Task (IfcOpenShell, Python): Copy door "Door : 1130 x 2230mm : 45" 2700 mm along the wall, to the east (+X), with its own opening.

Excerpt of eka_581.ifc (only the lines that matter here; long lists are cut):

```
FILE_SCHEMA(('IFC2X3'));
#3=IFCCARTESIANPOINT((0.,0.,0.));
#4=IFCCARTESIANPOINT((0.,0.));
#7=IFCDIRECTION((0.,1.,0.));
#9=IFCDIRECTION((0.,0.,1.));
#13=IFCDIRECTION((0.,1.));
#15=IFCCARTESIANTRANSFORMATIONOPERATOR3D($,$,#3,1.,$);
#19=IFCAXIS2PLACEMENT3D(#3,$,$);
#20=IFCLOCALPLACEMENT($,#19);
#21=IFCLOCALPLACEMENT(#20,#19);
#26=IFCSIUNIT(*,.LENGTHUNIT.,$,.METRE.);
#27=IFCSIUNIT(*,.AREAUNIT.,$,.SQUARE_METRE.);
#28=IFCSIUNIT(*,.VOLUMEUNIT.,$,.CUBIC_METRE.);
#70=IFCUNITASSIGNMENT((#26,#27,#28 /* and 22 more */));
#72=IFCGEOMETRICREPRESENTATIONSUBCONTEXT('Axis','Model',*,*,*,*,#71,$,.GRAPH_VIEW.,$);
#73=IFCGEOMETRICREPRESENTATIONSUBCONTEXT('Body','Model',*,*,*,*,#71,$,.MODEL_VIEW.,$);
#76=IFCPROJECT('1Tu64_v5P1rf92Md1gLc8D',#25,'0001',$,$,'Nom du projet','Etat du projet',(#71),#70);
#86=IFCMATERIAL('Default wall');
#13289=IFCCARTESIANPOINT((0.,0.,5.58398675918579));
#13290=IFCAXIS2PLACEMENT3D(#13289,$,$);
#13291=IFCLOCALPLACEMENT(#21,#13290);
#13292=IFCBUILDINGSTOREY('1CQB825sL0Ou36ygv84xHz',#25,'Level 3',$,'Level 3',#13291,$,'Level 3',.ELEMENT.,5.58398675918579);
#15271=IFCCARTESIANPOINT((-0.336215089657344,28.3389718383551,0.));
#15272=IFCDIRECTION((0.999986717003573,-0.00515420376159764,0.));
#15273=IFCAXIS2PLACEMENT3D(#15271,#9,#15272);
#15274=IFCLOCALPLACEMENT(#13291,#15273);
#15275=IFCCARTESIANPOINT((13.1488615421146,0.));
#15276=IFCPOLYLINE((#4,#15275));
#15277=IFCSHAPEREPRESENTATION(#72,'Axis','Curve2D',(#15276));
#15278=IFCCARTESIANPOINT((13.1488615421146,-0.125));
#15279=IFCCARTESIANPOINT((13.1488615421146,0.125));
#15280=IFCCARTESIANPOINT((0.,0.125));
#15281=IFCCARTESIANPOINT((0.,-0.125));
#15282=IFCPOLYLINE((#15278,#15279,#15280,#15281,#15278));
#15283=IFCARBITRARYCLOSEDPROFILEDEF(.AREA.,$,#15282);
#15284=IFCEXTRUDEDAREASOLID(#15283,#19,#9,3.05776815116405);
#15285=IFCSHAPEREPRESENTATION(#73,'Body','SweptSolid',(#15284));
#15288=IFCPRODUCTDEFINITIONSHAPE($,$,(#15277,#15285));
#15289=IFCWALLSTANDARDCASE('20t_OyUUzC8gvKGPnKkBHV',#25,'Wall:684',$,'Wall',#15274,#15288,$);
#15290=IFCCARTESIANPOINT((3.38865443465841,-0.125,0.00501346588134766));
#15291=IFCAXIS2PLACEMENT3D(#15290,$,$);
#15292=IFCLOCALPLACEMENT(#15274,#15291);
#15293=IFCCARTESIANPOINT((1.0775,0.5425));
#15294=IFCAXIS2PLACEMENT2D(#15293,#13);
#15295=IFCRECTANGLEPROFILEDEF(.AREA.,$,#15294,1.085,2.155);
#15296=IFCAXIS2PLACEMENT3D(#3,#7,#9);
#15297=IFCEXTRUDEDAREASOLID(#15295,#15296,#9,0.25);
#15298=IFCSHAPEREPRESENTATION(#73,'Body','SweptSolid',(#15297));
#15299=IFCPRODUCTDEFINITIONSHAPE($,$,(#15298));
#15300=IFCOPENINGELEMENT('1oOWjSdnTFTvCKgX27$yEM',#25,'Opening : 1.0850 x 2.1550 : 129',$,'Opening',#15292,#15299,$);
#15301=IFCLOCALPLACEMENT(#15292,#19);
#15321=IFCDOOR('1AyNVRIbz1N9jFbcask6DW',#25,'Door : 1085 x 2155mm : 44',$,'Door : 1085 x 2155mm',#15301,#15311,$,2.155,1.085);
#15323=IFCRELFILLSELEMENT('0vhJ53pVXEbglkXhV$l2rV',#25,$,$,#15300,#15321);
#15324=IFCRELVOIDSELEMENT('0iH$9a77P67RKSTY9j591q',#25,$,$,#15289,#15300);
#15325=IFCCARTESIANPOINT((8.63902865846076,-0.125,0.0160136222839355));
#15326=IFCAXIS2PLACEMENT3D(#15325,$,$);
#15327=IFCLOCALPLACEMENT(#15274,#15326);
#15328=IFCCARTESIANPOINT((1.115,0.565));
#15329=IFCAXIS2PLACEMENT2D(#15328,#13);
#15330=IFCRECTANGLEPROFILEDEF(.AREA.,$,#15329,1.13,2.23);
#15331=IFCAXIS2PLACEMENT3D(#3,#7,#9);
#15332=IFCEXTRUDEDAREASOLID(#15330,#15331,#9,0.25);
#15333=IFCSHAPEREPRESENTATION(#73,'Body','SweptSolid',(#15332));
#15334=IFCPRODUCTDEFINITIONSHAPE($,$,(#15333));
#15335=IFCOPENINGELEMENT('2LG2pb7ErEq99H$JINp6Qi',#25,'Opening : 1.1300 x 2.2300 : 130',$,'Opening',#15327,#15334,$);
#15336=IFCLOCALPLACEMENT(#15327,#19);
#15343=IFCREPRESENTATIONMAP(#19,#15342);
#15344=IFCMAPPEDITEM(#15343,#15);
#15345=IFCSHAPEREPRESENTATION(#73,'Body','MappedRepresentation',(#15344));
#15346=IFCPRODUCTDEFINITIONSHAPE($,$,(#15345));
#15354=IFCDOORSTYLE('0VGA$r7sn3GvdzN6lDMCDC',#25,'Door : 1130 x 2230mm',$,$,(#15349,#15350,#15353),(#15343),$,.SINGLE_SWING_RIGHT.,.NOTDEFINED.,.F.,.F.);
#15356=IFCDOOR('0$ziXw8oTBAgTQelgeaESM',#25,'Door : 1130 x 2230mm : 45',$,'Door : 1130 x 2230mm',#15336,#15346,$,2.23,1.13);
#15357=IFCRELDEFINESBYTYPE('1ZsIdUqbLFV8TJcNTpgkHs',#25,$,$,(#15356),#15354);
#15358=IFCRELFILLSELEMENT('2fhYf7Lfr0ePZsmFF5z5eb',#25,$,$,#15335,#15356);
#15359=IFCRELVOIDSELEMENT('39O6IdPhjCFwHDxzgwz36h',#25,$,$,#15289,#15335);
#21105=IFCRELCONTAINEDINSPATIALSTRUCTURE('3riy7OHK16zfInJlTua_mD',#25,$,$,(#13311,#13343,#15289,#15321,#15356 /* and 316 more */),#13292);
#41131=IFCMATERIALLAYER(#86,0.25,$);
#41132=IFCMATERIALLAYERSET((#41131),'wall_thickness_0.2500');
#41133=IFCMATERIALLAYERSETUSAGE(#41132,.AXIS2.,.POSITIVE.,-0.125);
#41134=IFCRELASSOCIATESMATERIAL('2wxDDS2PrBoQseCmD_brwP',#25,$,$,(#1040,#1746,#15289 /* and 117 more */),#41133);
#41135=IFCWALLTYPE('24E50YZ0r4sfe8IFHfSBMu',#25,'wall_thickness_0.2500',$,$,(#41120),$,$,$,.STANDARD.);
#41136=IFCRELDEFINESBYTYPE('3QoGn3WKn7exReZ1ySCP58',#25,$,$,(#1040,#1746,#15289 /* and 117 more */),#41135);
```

```python
import ifcopenshell
import ifcopenshell.api.feature
import ifcopenshell.api.geometry
import ifcopenshell.api.root
import ifcopenshell.geom
import ifcopenshell.util.element
import ifcopenshell.util.placement
import ifcopenshell.util.shape

model = ifcopenshell.open("eka_581.ifc")
settings = ifcopenshell.geom.settings()


def volume(element):
    """Net volume in cubic metres, openings subtracted."""
    shape = ifcopenshell.geom.create_shape(settings, element)
    return ifcopenshell.util.shape.get_volume(shape.geometry)


door = model.by_id(15356)
opening = door.FillsVoids[0].RelatingOpeningElement
wall = opening.VoidsElements[0].RelatingBuildingElement
before = volume(wall)
shift = ifcopenshell.util.placement.get_local_placement(wall.ObjectPlacement)[:3, 0] * 2.7

# copy_class copies the void relationship, type, container and properties, but no geometry.
new_opening = ifcopenshell.api.root.copy_class(model, product=opening)
new_opening.Representation = ifcopenshell.util.element.copy_deep(
    model, opening.Representation, exclude=["IfcGeometricRepresentationContext", "IfcRepresentationMap"]
)
new_opening.Name = "Opening : 1.1300 x 2.2300"
new_door = ifcopenshell.api.root.copy_class(model, product=door)
new_door.Representation = ifcopenshell.util.element.copy_deep(
    model, door.Representation, exclude=["IfcGeometricRepresentationContext", "IfcRepresentationMap"]
)
new_door.Name = "Door : 1130 x 2230mm"
fills = ifcopenshell.api.feature.add_filling(model, opening=new_opening, element=new_door)
fills.OwnerHistory = new_door.OwnerHistory  # required in IFC2X3

for old, new in ((opening, new_opening), (door, new_door)):
    matrix = ifcopenshell.util.placement.get_local_placement(old.ObjectPlacement)
    matrix[:3, 3] += shift
    ifcopenshell.api.geometry.edit_object_placement(model, product=new, matrix=matrix, is_si=False)

after = volume(wall)

print(f"wall volume {before:.3f} -> {after:.3f} m3")

model.write("eka_581_edited.ifc")
```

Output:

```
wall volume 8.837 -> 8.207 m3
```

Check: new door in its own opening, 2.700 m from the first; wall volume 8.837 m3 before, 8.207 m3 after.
